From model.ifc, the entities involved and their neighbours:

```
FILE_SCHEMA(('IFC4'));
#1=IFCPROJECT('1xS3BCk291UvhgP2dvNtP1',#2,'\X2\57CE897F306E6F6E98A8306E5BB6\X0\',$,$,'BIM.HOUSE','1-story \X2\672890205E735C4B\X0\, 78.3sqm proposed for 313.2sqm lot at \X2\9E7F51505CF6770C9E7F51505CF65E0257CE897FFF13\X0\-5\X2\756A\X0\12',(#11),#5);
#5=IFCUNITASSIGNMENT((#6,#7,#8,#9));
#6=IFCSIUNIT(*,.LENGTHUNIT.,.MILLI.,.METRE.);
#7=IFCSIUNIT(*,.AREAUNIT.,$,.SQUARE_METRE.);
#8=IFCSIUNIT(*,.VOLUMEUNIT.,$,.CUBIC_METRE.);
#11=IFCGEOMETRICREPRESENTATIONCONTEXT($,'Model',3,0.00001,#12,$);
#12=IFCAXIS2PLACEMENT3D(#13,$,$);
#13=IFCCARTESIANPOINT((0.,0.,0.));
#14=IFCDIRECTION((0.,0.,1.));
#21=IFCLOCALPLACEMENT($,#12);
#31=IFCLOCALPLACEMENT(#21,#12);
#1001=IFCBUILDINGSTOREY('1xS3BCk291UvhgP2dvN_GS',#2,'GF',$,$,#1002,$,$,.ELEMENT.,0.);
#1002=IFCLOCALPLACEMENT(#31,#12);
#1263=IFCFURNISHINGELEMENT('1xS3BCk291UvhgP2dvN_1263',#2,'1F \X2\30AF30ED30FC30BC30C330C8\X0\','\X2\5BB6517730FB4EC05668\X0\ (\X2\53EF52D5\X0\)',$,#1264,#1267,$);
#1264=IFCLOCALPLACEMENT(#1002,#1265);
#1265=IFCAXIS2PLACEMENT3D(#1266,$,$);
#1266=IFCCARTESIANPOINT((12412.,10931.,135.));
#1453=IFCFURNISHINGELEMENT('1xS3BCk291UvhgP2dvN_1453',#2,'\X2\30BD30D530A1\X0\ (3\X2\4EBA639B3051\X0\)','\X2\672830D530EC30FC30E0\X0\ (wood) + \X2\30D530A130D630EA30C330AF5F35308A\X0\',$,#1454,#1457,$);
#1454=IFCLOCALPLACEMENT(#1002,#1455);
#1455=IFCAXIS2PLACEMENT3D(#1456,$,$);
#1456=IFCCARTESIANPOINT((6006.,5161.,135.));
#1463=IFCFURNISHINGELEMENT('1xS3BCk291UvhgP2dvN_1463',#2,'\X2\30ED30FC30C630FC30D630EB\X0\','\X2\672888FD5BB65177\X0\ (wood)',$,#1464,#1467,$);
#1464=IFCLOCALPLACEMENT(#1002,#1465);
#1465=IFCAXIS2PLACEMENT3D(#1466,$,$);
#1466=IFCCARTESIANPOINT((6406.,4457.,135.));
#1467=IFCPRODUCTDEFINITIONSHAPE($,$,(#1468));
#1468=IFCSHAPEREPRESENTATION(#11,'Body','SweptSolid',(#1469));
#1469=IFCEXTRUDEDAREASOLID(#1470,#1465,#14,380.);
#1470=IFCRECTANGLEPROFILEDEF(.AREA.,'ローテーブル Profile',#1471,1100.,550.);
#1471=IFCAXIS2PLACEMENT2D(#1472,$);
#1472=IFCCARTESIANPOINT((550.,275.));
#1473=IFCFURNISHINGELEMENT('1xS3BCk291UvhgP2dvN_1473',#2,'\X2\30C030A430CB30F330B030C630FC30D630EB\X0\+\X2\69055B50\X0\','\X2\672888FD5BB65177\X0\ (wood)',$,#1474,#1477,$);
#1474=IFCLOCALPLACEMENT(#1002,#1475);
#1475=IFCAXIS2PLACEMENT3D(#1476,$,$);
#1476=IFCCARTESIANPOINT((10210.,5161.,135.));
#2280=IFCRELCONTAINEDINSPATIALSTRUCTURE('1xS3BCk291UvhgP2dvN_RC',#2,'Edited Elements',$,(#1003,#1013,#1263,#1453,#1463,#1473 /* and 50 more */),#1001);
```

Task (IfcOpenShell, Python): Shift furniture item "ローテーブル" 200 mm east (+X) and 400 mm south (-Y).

```python
import ifcopenshell
import ifcopenshell.api.geometry
import ifcopenshell.util.placement
import ifcopenshell.util.unit

model = ifcopenshell.open("model.ifc")
unit_scale = ifcopenshell.util.unit.calculate_unit_scale(model)

item = model.by_guid("1xS3BCk291UvhgP2dvN_1463")
matrix = ifcopenshell.util.placement.get_local_placement(item.ObjectPlacement)
matrix[0, 3] += 0.2 / unit_scale
matrix[1, 3] -= 0.4 / unit_scale
ifcopenshell.api.geometry.edit_object_placement(model, product=item, matrix=matrix, is_si=False)

print(ifcopenshell.util.placement.get_local_placement(item.ObjectPlacement).round(3) + 0.0)

model.write("model_v2.ifc")
```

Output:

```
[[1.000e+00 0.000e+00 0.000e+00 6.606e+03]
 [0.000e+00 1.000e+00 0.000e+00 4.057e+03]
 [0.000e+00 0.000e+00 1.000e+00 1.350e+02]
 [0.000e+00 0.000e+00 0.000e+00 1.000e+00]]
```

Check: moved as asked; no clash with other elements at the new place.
